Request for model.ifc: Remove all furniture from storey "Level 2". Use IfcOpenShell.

First a look at what the model holds.

```python
import ifcopenshell
import ifcopenshell.util.element

model = ifcopenshell.open("model.ifc")
print(model.schema)
storey = next(s for s in model.by_type("IfcBuildingStorey") if s.Name == "Level 2")
furniture = [e for e in ifcopenshell.util.element.get_decomposition(storey) if e.is_a("IfcFurnishingElement")]
seen = {}
for e in furniture:
    element_type = ifcopenshell.util.element.get_type(e)
    name = element_type.Name if element_type not in (None, e) else None
    seen[name] = seen.get(name, 0) + 1
for name, count in sorted(seen.items(), key=str):
    print(count, "x", name)
```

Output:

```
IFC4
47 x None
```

```python
import ifcopenshell
import ifcopenshell.api.root
import ifcopenshell.util.element

model = ifcopenshell.open("model.ifc")

storey = next(s for s in model.by_type("IfcBuildingStorey") if s.Name == "Level 2")
furniture = [e for e in ifcopenshell.util.element.get_decomposition(storey) if e.is_a("IfcFurnishingElement")]

for e in furniture:
    ifcopenshell.api.root.remove_product(model, product=e)
print(len(furniture), "removed")

model.write("model_rev.ifc")
```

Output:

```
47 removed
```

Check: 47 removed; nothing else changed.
